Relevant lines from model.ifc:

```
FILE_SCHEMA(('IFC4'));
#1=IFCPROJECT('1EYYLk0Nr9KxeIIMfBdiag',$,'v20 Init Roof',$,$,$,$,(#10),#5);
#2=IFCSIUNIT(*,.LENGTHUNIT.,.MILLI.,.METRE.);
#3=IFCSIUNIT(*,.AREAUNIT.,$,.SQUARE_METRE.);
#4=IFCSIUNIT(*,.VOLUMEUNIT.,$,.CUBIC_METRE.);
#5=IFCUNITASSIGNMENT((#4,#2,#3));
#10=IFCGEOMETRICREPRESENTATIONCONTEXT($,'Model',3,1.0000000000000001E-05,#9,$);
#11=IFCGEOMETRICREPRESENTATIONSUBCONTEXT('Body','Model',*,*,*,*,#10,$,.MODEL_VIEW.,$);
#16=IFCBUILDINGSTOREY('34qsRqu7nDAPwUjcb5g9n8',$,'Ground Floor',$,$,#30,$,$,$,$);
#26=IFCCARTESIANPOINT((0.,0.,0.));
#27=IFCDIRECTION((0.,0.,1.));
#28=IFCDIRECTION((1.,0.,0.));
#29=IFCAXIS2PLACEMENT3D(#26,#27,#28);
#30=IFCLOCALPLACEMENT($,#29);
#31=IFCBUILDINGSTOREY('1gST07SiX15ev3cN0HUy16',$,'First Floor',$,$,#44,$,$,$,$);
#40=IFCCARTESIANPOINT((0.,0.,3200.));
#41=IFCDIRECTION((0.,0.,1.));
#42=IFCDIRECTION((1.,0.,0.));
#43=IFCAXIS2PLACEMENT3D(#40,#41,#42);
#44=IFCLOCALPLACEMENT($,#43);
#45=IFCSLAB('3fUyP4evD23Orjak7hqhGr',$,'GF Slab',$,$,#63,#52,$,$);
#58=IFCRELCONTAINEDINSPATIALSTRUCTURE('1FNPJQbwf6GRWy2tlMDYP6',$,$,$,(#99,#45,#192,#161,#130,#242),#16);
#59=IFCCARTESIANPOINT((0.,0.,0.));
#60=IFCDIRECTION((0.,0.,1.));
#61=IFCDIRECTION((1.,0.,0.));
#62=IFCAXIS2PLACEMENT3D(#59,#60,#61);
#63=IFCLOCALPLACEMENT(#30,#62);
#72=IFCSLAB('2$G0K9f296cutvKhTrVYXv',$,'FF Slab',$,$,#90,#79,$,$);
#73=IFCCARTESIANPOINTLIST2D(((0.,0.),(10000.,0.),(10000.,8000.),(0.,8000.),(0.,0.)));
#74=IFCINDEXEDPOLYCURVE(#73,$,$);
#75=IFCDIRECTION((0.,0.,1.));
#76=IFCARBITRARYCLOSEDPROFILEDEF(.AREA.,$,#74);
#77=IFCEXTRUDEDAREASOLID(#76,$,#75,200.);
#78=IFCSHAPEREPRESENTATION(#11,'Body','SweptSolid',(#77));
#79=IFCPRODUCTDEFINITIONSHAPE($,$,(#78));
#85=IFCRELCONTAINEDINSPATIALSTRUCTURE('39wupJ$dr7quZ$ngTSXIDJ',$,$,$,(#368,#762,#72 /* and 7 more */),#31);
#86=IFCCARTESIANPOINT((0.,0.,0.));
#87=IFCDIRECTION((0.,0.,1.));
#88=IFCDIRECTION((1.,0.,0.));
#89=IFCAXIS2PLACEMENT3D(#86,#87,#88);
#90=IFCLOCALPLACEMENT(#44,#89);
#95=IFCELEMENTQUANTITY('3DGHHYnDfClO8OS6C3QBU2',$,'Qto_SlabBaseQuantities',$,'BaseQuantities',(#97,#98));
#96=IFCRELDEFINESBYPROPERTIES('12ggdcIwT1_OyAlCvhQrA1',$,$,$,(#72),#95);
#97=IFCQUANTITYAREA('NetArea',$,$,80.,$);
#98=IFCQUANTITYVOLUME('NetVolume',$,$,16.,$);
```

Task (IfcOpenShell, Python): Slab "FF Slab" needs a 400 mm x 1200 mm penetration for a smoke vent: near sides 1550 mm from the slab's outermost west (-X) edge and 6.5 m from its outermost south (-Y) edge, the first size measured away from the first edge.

```python
import numpy as np
import ifcopenshell
import ifcopenshell.api.feature
import ifcopenshell.api.geometry
import ifcopenshell.api.pset
import ifcopenshell.api.root
import ifcopenshell.geom
import ifcopenshell.util.element
import ifcopenshell.util.placement
import ifcopenshell.util.representation
import ifcopenshell.util.shape
import ifcopenshell.util.unit

model = ifcopenshell.open("model.ifc")
unit_scale = ifcopenshell.util.unit.calculate_unit_scale(model)
area_scale = ifcopenshell.util.unit.calculate_unit_scale(model, "AREAUNIT")
volume_scale = ifcopenshell.util.unit.calculate_unit_scale(model, "VOLUMEUNIT")
settings = ifcopenshell.geom.settings()


def volume(element):
    """Net volume in cubic metres, openings subtracted."""
    shape = ifcopenshell.geom.create_shape(settings, element)
    return ifcopenshell.util.shape.get_volume(shape.geometry)


slab = model.by_guid("2$G0K9f296cutvKhTrVYXv")
before = volume(slab)

# Extent in the slab's own axes, in metres. The edges named are its -X and -Y sides.
slab_shape = ifcopenshell.geom.create_shape(settings, slab)
vertices = ifcopenshell.util.shape.get_vertices(slab_shape.geometry)
x_min, y_min, bottom = vertices.min(axis=0)
top = vertices[:, 2].max()

opening = ifcopenshell.api.root.create_entity(model, ifc_class="IfcOpeningElement", name="Smoke vent opening", predefined_type="OPENING")
context = ifcopenshell.util.representation.get_context(model, "Model", "Body", "MODEL_VIEW")
width, depth = 0.4, 1.2
outline = [(0.0, 0.0), (width, 0.0), (width, depth), (0.0, depth), (0.0, 0.0)]
# Overshoot both faces by 50 mm so the cut is clean.
shape = ifcopenshell.api.geometry.add_slab_representation(
    model, context=context, depth=top - bottom + 0.1, polyline=outline
)
ifcopenshell.api.geometry.assign_representation(model, product=opening, representation=shape)

matrix = ifcopenshell.util.placement.get_local_placement(slab.ObjectPlacement)
matrix[:, 3] = matrix @ np.append(np.array([x_min + 1.55, y_min + 6.5, bottom - 0.05]) / unit_scale, 1.0)
ifcopenshell.api.geometry.edit_object_placement(model, product=opening, matrix=matrix, is_si=False)
ifcopenshell.api.feature.add_feature(model, feature=opening, element=slab)

after = volume(slab)

# Update the slab's stored quantities.
qto = model.by_id(ifcopenshell.util.element.get_pset(slab, "Qto_SlabBaseQuantities", should_inherit=False)["id"])
ifcopenshell.api.pset.edit_qto(model, qto=qto, properties={
    "NetArea": after / (top - bottom) / area_scale,
    "NetVolume": after / volume_scale,
})

print(f"slab volume {before:.3f} -> {after:.3f} m3")

model.write("model_edited.ifc")
```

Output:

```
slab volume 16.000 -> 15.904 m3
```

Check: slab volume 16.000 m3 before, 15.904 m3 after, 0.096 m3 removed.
